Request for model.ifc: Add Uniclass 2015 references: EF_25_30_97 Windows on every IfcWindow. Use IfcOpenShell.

First a look at what the model holds.

```python
import ifcopenshell

model = ifcopenshell.open("model.ifc")
print(model.schema)
print("classifications:", [c.Name for c in model.by_type("IfcClassification")])
for ifc_class in ("IfcDoor", "IfcRoof", "IfcStair", "IfcWall", "IfcWindow"):
    print(ifc_class, len(model.by_type(ifc_class)))
```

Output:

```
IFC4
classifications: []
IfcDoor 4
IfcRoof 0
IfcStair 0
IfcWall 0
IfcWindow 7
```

```python
import ifcopenshell
import ifcopenshell.api.classification

model = ifcopenshell.open("model.ifc")

system = ifcopenshell.api.classification.add_classification(model, classification="Uniclass 2015")

codes = {
    "IfcWindow": ("EF_25_30_97", "Windows"),
}
for ifc_class, (code, name) in codes.items():
    products = model.by_type(ifc_class)
    ifcopenshell.api.classification.add_reference(
        model, products=products, classification=system, identification=code, name=name
    )
    print(code, len(products))

model.write("model_edited.ifc")
```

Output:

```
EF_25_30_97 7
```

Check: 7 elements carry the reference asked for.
